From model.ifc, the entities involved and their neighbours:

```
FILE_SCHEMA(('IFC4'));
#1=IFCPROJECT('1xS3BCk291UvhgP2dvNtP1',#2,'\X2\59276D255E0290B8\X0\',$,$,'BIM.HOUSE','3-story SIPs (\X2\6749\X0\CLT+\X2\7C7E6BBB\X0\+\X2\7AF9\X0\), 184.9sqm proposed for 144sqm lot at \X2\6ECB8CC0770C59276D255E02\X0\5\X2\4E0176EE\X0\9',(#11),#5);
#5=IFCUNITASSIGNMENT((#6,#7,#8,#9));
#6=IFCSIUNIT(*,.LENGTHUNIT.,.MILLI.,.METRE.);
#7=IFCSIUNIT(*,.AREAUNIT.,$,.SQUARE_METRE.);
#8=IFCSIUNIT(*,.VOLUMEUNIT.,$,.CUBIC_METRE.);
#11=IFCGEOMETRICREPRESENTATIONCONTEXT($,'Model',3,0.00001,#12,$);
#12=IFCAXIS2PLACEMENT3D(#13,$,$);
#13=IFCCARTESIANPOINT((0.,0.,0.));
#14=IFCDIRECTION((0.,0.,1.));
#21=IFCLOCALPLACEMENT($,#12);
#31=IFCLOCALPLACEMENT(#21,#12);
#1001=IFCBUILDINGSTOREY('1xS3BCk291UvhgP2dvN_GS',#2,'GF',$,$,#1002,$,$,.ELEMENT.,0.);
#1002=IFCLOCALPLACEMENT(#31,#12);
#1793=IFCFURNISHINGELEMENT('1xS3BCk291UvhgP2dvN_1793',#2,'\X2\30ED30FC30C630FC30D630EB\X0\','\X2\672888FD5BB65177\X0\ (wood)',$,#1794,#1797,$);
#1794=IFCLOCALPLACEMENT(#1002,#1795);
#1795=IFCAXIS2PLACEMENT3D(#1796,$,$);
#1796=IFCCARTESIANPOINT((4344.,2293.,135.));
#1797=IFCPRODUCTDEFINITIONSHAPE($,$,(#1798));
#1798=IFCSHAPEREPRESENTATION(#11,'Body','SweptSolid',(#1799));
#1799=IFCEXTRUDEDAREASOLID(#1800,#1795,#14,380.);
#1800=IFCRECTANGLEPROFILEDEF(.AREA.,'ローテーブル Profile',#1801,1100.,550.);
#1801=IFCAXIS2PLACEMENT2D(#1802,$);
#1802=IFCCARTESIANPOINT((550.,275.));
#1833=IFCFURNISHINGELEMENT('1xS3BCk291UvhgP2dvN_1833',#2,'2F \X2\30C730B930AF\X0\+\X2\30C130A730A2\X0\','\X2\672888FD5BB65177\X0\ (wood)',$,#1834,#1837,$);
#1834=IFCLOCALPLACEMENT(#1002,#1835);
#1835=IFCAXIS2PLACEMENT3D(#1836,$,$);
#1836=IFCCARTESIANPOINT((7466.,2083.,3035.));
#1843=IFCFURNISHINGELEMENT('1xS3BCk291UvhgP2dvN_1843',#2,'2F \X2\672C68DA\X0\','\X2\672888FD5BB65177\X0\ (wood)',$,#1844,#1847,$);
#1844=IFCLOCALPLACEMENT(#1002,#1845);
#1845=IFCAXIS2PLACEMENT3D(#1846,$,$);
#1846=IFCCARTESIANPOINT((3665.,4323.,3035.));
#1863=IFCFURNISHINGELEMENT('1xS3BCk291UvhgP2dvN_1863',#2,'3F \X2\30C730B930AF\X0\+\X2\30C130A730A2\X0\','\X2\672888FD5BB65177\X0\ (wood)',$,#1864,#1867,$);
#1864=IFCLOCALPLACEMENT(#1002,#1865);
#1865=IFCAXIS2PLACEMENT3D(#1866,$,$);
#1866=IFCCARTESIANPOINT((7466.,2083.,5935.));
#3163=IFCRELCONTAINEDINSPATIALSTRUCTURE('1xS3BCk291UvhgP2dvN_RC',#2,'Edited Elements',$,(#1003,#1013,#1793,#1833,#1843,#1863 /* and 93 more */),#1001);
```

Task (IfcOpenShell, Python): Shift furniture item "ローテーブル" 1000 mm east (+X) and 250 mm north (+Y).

```python
import ifcopenshell
import ifcopenshell.api.geometry
import ifcopenshell.util.placement
import ifcopenshell.util.unit

model = ifcopenshell.open("model.ifc")
unit_scale = ifcopenshell.util.unit.calculate_unit_scale(model)

item = model.by_guid("1xS3BCk291UvhgP2dvN_1793")
matrix = ifcopenshell.util.placement.get_local_placement(item.ObjectPlacement)
matrix[0, 3] += 1 / unit_scale
matrix[1, 3] += 0.25 / unit_scale
ifcopenshell.api.geometry.edit_object_placement(model, product=item, matrix=matrix, is_si=False)

print(ifcopenshell.util.placement.get_local_placement(item.ObjectPlacement).round(3) + 0.0)

model.write("model_updated.ifc")
```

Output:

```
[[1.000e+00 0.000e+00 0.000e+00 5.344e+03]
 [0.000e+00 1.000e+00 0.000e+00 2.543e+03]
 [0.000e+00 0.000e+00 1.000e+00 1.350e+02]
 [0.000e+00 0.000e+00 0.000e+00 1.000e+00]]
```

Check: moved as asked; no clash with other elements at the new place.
